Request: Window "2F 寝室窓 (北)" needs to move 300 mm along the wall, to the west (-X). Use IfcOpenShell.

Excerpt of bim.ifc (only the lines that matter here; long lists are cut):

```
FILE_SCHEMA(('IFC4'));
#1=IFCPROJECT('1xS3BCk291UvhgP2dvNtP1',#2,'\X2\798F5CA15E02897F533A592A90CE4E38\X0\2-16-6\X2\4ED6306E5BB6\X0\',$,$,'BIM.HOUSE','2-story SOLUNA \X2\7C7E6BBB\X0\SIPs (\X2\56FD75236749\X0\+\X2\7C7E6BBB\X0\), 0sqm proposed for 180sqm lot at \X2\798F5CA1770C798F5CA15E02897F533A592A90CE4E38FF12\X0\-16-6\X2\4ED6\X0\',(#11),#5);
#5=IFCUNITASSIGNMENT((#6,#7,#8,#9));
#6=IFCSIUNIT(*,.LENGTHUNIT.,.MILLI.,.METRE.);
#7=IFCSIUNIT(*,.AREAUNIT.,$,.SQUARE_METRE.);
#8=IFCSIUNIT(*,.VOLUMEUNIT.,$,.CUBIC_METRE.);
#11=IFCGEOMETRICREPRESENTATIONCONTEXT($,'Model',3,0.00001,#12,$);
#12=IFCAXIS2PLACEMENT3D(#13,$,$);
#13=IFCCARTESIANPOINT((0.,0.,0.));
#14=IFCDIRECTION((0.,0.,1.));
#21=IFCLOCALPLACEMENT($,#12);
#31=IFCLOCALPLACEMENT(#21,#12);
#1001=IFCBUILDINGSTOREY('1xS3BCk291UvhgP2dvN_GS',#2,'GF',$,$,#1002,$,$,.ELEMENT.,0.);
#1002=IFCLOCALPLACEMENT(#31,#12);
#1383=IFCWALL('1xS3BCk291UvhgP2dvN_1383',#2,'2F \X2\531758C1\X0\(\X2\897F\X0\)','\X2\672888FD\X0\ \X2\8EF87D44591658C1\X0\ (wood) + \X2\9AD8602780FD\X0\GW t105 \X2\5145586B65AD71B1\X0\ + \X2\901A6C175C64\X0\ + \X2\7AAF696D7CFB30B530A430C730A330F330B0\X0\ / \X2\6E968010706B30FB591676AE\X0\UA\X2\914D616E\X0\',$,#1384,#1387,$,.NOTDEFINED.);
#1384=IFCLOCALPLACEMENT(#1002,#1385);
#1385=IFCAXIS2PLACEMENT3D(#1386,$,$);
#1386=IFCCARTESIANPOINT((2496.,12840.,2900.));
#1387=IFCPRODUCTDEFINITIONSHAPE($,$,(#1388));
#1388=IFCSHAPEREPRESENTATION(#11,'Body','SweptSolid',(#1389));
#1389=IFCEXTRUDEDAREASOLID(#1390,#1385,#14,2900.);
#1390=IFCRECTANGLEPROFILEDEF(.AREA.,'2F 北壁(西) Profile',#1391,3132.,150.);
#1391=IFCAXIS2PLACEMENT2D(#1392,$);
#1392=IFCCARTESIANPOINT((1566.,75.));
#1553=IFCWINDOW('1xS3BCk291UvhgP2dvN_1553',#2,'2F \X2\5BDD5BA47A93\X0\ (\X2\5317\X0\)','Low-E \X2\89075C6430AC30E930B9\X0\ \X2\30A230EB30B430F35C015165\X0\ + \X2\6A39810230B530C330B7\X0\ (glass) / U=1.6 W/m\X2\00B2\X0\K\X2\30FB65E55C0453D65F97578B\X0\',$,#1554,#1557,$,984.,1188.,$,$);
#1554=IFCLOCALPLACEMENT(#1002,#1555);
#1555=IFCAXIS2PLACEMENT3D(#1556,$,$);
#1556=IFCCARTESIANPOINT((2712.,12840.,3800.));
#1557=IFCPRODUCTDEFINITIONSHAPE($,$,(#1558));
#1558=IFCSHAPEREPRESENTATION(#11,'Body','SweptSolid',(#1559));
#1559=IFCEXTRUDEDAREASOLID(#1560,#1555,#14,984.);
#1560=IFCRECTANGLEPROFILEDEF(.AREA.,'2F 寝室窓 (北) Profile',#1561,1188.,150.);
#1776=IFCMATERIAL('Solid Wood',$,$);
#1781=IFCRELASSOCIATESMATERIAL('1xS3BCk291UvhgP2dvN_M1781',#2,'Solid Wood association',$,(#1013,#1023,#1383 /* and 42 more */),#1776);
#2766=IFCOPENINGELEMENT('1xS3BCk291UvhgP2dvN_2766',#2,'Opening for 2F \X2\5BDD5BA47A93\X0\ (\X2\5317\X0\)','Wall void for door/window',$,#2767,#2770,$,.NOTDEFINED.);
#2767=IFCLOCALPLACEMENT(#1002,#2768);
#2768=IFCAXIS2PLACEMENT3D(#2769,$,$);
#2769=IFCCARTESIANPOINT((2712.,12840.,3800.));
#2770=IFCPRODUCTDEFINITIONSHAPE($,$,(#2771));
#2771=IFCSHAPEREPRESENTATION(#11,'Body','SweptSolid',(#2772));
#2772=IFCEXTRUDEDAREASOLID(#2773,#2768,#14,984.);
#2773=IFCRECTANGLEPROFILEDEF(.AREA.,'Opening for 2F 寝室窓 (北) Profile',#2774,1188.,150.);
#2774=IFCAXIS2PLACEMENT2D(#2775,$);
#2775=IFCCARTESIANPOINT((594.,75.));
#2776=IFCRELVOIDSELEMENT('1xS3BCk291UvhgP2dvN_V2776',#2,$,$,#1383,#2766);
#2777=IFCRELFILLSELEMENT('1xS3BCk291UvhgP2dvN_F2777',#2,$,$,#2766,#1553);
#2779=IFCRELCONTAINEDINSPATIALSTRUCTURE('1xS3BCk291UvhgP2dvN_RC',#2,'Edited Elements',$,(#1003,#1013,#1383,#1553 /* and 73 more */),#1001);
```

```python
import ifcopenshell
import ifcopenshell.api.geometry
import ifcopenshell.util.placement
import ifcopenshell.util.unit

model = ifcopenshell.open("bim.ifc")
unit_scale = ifcopenshell.util.unit.calculate_unit_scale(model)

window = model.by_guid("1xS3BCk291UvhgP2dvN_1553")
opening = window.FillsVoids[0].RelatingOpeningElement
wall = opening.VoidsElements[0].RelatingBuildingElement

wall_matrix = ifcopenshell.util.placement.get_local_placement(wall.ObjectPlacement)
shift = wall_matrix[:3, 0] * -0.3 / unit_scale
before = ifcopenshell.util.placement.get_local_placement(window.ObjectPlacement)[:3, 3].copy()

# The window is not placed relative to its opening, so move both.
for product in (opening, window):
    matrix = ifcopenshell.util.placement.get_local_placement(product.ObjectPlacement)
    matrix[:3, 3] += shift
    ifcopenshell.api.geometry.edit_object_placement(model, product=product, matrix=matrix, is_si=False)

after = ifcopenshell.util.placement.get_local_placement(window.ObjectPlacement)[:3, 3]
print("window moved by", (after - before).round(3) + 0.0)

model.write("bim_v2.ifc")
```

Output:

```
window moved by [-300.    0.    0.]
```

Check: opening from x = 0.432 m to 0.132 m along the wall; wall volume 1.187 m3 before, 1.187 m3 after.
